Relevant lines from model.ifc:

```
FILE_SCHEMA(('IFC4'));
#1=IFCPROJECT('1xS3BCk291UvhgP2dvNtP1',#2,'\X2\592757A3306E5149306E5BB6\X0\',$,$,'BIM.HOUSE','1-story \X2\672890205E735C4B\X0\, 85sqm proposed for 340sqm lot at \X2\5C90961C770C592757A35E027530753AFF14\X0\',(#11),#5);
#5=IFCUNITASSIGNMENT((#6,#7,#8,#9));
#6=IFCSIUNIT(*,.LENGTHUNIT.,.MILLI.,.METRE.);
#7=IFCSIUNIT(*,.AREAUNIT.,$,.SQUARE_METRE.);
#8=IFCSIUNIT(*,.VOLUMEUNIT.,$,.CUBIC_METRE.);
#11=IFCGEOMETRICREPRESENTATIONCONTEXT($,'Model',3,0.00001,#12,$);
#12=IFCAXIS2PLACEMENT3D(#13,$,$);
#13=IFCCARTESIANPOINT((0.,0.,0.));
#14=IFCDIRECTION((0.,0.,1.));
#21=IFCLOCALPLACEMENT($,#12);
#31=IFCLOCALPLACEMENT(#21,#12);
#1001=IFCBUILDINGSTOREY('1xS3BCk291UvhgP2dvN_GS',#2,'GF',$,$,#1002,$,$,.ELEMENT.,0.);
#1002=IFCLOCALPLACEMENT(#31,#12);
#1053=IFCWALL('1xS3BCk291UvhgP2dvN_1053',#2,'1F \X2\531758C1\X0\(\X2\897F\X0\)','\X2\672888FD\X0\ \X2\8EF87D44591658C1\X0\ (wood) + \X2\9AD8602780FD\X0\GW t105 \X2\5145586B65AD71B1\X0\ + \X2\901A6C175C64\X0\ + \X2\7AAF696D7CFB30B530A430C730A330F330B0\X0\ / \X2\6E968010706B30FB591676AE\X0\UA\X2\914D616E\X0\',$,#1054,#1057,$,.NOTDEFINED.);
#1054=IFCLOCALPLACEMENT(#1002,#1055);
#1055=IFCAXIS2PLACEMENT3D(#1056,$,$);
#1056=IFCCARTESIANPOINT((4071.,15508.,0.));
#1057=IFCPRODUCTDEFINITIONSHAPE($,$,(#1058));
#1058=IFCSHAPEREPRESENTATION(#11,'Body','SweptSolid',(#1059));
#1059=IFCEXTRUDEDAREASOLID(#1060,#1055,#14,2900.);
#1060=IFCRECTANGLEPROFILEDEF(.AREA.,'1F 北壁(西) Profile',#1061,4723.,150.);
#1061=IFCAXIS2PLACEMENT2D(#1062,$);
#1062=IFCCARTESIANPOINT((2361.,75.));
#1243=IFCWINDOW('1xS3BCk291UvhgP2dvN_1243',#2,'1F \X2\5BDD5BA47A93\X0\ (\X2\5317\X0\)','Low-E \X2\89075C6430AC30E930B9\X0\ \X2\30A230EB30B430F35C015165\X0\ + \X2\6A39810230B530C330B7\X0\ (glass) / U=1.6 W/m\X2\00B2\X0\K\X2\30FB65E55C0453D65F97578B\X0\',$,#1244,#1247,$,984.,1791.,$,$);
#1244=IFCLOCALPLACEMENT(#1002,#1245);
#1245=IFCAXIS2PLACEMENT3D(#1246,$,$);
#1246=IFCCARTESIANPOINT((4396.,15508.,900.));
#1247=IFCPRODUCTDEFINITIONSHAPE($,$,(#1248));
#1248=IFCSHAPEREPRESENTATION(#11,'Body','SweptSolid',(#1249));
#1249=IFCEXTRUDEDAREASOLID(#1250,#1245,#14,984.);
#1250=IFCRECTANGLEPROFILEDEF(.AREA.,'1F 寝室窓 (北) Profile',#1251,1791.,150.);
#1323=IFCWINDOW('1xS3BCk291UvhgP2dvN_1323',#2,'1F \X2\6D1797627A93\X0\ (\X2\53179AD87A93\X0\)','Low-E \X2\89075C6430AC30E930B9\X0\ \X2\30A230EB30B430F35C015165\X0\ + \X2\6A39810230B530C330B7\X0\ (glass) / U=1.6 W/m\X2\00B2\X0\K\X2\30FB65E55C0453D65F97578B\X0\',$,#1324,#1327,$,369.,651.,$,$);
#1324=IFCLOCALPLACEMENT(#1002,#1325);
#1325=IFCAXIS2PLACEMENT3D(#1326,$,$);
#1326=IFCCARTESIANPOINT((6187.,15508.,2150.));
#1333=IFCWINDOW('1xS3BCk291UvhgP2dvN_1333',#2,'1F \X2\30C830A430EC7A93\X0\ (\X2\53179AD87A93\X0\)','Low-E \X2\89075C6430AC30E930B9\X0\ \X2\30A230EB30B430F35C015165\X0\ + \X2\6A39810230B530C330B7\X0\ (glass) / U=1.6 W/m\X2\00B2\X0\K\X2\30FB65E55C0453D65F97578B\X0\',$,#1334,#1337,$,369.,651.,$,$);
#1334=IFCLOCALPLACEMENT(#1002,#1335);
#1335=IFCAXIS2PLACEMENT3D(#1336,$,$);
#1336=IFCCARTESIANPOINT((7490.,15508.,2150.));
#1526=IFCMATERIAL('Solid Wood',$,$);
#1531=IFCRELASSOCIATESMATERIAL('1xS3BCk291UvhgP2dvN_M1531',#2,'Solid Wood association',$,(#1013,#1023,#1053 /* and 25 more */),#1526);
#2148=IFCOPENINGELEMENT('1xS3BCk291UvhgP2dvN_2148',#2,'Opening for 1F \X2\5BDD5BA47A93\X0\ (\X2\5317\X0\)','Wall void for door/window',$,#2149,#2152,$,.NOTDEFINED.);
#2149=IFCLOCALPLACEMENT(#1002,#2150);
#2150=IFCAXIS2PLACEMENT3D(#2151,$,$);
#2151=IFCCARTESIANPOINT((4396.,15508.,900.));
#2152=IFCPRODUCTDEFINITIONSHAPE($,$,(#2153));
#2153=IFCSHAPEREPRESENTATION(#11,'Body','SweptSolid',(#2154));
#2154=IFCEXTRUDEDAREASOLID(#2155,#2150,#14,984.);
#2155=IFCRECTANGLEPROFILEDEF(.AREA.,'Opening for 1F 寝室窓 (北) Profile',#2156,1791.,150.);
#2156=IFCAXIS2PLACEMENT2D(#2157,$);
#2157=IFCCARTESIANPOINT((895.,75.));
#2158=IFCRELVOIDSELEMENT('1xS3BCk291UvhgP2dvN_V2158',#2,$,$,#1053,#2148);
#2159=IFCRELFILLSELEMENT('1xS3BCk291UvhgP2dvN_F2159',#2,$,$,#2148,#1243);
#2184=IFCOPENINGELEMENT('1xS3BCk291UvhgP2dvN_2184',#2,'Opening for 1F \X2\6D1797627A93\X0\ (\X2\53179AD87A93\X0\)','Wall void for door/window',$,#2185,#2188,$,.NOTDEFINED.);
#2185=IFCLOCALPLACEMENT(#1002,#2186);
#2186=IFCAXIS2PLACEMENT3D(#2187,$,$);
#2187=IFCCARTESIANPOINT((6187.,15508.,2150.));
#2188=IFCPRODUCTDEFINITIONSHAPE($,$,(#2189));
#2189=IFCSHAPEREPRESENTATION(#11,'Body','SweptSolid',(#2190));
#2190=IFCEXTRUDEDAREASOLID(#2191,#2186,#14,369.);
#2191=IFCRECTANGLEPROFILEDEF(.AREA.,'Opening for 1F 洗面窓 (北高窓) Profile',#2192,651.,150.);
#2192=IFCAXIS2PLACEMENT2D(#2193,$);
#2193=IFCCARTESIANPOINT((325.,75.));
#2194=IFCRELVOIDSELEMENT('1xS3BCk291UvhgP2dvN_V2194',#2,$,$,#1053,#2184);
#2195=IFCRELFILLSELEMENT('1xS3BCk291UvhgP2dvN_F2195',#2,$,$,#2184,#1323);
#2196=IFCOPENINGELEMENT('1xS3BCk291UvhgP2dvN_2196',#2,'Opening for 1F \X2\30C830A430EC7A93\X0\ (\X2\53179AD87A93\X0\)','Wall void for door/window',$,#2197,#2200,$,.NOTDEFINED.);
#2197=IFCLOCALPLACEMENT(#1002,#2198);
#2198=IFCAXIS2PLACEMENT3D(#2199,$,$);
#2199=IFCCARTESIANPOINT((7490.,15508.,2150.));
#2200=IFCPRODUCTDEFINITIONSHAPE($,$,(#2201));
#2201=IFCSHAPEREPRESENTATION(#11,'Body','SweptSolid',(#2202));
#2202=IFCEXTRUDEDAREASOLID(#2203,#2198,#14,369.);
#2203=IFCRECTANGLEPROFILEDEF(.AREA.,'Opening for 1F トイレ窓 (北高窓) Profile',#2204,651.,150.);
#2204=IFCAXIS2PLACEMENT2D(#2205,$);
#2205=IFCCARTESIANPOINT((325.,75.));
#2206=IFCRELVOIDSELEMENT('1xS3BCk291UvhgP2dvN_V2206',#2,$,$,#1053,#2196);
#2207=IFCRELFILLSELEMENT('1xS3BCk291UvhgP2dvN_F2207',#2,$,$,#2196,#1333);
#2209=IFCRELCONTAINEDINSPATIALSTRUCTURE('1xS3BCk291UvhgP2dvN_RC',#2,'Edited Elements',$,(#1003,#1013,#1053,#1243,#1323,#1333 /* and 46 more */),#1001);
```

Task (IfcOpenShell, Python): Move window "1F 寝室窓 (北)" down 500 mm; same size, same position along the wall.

```python
import numpy as np
import ifcopenshell
import ifcopenshell.api.geometry
import ifcopenshell.util.placement
import ifcopenshell.util.unit

model = ifcopenshell.open("model.ifc")
unit_scale = ifcopenshell.util.unit.calculate_unit_scale(model)

window = model.by_guid("1xS3BCk291UvhgP2dvN_1243")
opening = window.FillsVoids[0].RelatingOpeningElement
dz = -500.0

shift = np.array([0.0, 0.0, dz])
# The window is not placed relative to its opening, so move both.
for product in (opening, window):
    matrix = ifcopenshell.util.placement.get_local_placement(product.ObjectPlacement)
    matrix[:3, 3] += shift
    ifcopenshell.api.geometry.edit_object_placement(model, product=product, matrix=matrix, is_si=False)

print(f"moved by {dz * unit_scale:+.3f} m")

model.write("model_rev.ifc")
```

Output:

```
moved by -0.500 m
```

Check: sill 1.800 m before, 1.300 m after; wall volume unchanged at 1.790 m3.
